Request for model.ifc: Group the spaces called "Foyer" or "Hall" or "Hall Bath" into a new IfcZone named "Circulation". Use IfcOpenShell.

First a look at what the model holds.

```python
import ifcopenshell

model = ifcopenshell.open("model.ifc")
print(model.schema)
seen = {}
for space in model.by_type("IfcSpace"):
    seen[space.LongName] = seen.get(space.LongName, 0) + 1
for name, count in sorted(seen.items(), key=str):
    print(count, "x", name)
print("zones:", [z.Name for z in model.by_type("IfcZone")][:20])
```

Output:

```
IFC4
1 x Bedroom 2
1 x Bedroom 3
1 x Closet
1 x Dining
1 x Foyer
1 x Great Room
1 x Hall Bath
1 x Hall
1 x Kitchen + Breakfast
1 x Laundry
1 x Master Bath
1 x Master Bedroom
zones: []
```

```python
import ifcopenshell
import ifcopenshell.api.group
import ifcopenshell.api.root

model = ifcopenshell.open("model.ifc")

names = {"Foyer", "Hall", "Hall Bath"}
spaces = [s for s in model.by_type("IfcSpace") if s.LongName in names]

zone = ifcopenshell.api.root.create_entity(model, ifc_class="IfcZone", name="Circulation")
ifcopenshell.api.group.assign_group(model, products=spaces, group=zone)
print(len(spaces), "spaces in", zone.Name)

model.write("model-out.ifc")
```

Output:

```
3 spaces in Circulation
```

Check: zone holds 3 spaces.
